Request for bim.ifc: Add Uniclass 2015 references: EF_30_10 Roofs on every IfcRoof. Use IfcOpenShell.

First a look at what the model holds.

```python
import ifcopenshell

model = ifcopenshell.open("bim.ifc")
print(model.schema)
print("classifications:", [c.Name for c in model.by_type("IfcClassification")])
for ifc_class in ("IfcDoor", "IfcRoof", "IfcStair", "IfcWall", "IfcWindow"):
    print(ifc_class, len(model.by_type(ifc_class)))
```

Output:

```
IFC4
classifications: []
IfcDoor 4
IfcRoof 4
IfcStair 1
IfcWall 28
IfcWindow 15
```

```python
import ifcopenshell
import ifcopenshell.api.classification

model = ifcopenshell.open("bim.ifc")

system = ifcopenshell.api.classification.add_classification(model, classification="Uniclass 2015")

codes = {
    "IfcRoof": ("EF_30_10", "Roofs"),
}
for ifc_class, (code, name) in codes.items():
    products = model.by_type(ifc_class)
    ifcopenshell.api.classification.add_reference(
        model, products=products, classification=system, identification=code, name=name
    )
    print(code, len(products))

model.write("bim-out.ifc")
```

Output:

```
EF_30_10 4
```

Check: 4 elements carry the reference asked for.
